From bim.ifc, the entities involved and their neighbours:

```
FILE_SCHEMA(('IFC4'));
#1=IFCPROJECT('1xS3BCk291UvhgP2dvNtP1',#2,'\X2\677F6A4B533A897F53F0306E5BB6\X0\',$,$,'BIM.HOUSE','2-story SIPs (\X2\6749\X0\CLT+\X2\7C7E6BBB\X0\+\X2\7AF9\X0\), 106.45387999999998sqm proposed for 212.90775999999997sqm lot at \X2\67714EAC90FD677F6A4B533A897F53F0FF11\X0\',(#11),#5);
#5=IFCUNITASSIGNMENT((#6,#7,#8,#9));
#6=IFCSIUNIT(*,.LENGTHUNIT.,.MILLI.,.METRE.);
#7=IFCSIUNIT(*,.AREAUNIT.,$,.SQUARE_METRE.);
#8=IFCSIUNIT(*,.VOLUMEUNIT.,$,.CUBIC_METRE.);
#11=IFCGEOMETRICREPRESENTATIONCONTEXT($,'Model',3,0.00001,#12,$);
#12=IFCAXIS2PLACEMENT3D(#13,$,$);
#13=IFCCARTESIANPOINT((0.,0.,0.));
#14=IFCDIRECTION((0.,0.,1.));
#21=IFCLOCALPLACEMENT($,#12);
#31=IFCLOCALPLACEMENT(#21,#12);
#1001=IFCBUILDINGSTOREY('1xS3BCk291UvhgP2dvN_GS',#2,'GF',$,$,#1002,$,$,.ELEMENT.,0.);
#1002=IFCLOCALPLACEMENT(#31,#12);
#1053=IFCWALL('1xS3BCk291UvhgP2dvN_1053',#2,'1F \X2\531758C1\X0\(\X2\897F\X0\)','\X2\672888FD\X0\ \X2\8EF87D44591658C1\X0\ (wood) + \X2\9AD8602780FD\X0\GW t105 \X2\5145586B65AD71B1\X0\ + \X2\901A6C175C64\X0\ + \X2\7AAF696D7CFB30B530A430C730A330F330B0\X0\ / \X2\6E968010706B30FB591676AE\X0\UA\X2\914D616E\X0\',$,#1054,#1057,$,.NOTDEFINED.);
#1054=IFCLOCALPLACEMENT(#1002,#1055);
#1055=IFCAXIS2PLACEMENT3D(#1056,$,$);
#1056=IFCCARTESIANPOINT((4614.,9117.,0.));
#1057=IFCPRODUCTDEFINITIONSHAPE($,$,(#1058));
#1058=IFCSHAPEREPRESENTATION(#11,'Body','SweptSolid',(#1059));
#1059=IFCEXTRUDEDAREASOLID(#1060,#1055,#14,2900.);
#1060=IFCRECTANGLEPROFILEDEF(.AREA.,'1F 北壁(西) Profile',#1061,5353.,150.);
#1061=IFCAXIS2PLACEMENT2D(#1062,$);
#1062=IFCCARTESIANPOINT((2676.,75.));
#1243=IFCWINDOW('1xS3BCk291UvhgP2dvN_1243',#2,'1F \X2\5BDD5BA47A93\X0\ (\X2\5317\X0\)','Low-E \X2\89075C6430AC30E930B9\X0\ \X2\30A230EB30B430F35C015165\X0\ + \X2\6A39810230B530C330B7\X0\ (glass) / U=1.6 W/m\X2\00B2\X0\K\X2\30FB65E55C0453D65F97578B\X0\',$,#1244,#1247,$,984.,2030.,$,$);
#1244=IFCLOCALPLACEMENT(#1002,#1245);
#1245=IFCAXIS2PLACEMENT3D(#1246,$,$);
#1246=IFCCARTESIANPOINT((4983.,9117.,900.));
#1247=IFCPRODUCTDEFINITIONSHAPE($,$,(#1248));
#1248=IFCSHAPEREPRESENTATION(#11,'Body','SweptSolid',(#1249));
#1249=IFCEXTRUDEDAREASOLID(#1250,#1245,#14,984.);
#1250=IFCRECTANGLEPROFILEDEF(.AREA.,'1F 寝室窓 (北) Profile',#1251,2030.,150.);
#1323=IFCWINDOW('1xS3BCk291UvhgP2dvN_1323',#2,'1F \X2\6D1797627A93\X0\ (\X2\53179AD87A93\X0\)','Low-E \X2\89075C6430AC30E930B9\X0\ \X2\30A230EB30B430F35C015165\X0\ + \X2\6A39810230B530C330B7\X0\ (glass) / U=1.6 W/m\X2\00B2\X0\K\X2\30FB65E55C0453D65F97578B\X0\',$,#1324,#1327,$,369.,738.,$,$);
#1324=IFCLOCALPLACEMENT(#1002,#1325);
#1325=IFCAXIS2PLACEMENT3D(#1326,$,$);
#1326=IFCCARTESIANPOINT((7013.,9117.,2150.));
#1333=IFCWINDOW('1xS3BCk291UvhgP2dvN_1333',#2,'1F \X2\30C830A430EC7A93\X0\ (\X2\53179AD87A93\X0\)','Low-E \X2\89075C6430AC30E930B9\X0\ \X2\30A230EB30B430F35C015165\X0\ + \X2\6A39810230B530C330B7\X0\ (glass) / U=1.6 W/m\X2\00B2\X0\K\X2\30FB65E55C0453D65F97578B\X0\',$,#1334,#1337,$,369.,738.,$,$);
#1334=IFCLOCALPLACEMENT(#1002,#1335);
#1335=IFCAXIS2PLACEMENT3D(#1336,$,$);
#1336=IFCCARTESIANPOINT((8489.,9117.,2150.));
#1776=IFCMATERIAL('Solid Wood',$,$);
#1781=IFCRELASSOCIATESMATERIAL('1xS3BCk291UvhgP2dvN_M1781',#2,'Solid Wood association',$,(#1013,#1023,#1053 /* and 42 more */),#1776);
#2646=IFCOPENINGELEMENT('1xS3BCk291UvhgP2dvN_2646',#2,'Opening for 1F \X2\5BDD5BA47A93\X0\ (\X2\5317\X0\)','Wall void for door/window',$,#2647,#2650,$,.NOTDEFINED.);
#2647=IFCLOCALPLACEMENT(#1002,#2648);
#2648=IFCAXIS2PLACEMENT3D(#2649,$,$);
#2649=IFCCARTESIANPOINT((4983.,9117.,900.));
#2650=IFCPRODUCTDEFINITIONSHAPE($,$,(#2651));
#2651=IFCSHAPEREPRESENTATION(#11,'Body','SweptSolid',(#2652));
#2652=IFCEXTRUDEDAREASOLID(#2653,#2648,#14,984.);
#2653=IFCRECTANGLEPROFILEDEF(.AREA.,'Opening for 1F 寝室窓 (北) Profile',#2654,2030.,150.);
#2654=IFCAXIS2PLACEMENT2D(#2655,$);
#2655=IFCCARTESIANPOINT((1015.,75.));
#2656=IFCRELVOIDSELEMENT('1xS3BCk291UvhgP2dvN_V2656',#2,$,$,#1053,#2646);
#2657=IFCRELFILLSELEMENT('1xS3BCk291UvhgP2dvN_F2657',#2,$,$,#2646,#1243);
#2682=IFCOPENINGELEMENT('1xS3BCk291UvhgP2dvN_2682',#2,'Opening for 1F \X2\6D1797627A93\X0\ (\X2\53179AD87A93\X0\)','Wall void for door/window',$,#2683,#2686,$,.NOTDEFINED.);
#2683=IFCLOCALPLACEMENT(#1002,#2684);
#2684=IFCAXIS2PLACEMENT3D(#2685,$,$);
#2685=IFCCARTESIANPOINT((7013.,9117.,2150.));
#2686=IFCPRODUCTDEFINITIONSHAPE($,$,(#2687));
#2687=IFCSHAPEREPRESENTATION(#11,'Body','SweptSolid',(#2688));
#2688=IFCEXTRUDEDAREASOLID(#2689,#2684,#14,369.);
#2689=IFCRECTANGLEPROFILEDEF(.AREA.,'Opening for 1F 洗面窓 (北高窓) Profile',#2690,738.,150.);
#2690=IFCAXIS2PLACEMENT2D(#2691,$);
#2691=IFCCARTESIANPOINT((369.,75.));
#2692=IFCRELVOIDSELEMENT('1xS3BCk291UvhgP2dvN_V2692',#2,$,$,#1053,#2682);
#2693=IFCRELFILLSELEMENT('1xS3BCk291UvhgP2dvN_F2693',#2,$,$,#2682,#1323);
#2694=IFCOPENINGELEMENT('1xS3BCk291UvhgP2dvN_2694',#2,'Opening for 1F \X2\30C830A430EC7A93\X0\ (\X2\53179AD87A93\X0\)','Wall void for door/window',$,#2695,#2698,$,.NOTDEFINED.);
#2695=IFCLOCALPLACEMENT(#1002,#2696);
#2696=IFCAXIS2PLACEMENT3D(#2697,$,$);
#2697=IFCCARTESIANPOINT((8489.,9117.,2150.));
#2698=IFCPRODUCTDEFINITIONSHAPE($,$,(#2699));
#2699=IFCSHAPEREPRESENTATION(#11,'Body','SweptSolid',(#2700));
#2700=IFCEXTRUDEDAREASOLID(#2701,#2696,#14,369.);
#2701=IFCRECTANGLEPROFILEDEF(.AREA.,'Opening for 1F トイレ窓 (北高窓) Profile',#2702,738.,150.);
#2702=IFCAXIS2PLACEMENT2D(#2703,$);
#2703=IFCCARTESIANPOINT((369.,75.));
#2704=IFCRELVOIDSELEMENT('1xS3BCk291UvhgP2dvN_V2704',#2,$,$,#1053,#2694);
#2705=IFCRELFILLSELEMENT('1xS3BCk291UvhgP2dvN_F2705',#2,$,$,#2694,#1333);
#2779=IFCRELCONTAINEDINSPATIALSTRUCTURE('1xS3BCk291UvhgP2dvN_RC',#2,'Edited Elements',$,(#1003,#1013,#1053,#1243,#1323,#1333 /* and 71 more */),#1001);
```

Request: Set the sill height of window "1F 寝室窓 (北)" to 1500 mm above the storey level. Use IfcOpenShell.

```python
import numpy as np
import ifcopenshell
import ifcopenshell.api.geometry
import ifcopenshell.geom
import ifcopenshell.util.element
import ifcopenshell.util.placement
import ifcopenshell.util.shape
import ifcopenshell.util.unit

model = ifcopenshell.open("bim.ifc")
unit_scale = ifcopenshell.util.unit.calculate_unit_scale(model)

window = model.by_guid("1xS3BCk291UvhgP2dvN_1243")
opening = window.FillsVoids[0].RelatingOpeningElement
storey = ifcopenshell.util.element.get_container(window, ifc_class="IfcBuildingStorey")
level = ifcopenshell.util.placement.get_local_placement(storey.ObjectPlacement)[2, 3]

# The opening's origin need not be at the sill, so measure its lowest point.
shape = ifcopenshell.geom.create_shape(ifcopenshell.geom.settings(), opening)
bottom = ifcopenshell.util.shape.get_shape_bottom_elevation(shape, shape.geometry) / unit_scale
dz = level + 1.5 / unit_scale - bottom

shift = np.array([0.0, 0.0, dz])
# The window is not placed relative to its opening, so move both.
for product in (opening, window):
    matrix = ifcopenshell.util.placement.get_local_placement(product.ObjectPlacement)
    matrix[:3, 3] += shift
    ifcopenshell.api.geometry.edit_object_placement(model, product=product, matrix=matrix, is_si=False)

print(f"moved by {dz * unit_scale:+.3f} m")

model.write("bim_updated.ifc")
```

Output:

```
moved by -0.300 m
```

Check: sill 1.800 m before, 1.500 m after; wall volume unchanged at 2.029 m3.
